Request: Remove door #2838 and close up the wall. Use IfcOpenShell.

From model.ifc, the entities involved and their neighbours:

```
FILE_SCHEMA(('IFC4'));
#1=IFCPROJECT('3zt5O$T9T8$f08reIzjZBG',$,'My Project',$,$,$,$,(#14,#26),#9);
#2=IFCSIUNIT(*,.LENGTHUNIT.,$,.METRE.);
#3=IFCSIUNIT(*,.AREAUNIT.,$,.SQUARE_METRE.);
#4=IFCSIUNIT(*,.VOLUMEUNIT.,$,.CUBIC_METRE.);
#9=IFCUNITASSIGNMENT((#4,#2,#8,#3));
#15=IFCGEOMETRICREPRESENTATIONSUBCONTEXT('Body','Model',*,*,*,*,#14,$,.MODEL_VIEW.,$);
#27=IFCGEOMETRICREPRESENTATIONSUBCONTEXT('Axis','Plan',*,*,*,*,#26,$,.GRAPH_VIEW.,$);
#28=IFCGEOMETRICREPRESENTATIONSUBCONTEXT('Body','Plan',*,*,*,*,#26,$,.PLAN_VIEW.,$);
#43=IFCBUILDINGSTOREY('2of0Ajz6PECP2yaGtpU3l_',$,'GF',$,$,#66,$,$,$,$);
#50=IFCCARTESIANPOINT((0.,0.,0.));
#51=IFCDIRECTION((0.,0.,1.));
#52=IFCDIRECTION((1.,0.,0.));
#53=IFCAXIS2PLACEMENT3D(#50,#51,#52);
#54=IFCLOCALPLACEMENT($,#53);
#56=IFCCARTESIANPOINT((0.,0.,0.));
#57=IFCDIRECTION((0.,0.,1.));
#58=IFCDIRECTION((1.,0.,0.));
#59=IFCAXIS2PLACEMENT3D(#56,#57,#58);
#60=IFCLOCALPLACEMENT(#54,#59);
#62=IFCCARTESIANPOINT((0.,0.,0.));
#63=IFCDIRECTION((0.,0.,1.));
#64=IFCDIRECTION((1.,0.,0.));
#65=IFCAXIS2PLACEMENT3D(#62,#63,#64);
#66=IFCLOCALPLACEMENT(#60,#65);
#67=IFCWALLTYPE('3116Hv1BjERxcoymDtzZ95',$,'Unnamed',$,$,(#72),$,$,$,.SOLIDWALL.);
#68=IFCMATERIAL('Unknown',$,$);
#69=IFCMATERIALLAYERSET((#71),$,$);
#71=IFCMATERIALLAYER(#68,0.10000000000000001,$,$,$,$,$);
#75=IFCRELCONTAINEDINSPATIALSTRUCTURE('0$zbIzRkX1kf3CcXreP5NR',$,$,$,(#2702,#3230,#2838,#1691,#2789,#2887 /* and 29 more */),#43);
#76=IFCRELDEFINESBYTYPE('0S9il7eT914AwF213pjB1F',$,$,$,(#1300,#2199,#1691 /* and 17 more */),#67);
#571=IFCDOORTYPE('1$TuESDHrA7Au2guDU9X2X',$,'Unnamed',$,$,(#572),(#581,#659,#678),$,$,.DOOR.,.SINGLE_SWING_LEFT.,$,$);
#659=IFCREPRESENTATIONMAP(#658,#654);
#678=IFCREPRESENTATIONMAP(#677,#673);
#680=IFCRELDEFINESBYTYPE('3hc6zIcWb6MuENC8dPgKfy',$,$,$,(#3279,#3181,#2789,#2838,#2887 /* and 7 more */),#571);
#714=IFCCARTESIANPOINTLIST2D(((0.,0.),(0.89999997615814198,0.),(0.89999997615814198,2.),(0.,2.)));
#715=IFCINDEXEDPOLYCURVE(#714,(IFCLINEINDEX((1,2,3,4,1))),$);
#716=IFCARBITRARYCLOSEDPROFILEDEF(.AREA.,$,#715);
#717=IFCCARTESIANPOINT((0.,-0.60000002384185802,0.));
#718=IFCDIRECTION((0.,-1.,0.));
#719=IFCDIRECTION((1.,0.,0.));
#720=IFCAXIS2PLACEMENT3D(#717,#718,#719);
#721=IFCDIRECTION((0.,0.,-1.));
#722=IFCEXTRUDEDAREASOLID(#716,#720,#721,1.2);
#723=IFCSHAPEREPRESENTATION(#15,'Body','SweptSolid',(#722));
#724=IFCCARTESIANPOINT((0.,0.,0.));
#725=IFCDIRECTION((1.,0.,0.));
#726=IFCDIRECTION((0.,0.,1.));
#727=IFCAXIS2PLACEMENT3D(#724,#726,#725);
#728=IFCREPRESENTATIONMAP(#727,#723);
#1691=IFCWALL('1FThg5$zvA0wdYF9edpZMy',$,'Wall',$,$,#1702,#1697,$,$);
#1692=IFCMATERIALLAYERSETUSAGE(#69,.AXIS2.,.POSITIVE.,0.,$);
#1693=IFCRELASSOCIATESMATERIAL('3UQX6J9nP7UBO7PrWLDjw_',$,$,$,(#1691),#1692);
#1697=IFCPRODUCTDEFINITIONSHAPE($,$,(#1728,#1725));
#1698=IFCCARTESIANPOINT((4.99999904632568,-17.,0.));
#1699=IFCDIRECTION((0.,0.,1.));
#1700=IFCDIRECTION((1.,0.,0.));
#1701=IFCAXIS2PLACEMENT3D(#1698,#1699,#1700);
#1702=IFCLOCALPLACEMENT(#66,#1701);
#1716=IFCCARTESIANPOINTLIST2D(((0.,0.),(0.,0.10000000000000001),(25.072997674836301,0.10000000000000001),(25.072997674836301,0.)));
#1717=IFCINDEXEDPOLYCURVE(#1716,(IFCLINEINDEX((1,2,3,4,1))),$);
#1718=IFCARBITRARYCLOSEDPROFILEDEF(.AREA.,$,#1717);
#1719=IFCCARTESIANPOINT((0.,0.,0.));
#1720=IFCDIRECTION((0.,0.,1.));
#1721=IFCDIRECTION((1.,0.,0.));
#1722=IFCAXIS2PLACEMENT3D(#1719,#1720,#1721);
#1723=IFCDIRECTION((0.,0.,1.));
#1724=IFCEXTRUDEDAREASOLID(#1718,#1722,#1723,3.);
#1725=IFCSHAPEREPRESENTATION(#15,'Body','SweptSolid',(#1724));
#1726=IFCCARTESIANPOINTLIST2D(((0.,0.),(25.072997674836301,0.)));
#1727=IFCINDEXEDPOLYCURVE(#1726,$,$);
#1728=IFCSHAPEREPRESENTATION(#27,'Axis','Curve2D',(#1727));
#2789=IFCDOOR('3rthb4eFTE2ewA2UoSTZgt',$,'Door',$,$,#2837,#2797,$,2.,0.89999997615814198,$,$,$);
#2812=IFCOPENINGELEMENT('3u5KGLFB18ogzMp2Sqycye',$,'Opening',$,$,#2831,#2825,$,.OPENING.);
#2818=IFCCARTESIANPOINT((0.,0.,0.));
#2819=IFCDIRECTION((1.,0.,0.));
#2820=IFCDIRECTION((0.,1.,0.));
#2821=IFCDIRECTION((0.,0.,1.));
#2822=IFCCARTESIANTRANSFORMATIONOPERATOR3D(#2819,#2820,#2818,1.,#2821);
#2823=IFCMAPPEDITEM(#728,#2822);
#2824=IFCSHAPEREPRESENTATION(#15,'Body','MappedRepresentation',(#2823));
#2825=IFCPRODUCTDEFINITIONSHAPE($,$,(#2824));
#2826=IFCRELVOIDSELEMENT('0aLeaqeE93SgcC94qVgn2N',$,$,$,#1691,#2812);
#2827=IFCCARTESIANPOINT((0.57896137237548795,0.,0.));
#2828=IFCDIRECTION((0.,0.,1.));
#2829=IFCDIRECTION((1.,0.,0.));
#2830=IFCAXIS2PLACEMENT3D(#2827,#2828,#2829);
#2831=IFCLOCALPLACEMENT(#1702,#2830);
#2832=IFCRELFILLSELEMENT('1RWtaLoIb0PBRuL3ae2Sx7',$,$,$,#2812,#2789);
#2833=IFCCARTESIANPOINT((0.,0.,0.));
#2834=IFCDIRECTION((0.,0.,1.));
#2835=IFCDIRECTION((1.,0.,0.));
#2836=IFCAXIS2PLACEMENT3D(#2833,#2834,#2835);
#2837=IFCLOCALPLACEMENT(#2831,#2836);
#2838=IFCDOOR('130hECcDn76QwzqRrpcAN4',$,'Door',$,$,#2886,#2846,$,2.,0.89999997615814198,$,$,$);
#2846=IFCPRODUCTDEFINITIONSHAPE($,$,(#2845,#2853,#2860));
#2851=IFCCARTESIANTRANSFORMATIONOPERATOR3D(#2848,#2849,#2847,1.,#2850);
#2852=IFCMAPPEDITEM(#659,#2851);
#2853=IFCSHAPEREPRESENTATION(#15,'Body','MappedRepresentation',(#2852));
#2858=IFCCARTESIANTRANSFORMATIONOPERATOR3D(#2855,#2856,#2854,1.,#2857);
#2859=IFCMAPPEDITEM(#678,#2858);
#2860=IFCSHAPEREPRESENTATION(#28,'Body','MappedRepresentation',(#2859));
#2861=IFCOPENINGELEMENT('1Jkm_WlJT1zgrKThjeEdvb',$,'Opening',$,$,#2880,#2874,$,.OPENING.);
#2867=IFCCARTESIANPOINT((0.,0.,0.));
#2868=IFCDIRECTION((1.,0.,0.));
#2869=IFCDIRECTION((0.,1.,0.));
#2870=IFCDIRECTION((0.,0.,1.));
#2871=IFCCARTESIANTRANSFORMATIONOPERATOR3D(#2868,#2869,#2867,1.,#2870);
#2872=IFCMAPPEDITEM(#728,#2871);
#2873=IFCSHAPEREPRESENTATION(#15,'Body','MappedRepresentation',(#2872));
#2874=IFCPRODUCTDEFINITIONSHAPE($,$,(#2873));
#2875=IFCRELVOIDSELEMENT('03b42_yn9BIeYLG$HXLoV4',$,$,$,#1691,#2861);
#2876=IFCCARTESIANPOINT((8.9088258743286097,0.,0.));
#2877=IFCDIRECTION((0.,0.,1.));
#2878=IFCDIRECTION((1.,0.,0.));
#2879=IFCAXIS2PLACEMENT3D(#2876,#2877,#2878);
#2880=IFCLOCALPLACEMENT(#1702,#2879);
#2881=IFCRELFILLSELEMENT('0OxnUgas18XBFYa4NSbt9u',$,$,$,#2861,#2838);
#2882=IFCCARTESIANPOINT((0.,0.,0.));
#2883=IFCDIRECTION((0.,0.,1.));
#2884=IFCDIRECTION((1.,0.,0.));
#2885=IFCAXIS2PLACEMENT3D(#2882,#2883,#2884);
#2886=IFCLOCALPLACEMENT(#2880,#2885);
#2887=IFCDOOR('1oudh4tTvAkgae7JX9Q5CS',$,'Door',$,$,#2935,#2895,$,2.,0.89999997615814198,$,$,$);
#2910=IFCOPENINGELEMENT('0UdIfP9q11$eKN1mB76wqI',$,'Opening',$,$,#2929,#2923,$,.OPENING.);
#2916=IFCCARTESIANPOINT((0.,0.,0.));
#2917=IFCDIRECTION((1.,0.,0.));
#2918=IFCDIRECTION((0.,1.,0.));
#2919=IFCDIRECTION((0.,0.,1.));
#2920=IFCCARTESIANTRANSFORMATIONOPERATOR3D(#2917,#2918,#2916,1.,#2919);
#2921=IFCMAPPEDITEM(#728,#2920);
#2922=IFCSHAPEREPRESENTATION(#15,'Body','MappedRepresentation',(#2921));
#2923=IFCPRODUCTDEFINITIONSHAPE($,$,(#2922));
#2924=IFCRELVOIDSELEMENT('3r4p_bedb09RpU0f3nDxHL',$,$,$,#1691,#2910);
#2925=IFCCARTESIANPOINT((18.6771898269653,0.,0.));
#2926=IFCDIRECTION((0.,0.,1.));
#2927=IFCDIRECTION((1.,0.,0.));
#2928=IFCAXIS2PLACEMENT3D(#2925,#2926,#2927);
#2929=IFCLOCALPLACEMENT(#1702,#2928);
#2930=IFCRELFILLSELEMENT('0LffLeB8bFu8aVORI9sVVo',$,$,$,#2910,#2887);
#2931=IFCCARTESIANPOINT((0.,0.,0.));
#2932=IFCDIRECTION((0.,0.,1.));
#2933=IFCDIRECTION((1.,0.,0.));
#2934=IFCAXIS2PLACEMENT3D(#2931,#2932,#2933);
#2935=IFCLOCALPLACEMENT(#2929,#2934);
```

```python
import ifcopenshell
import ifcopenshell.api.feature
import ifcopenshell.api.root
import ifcopenshell.geom
import ifcopenshell.util.shape

model = ifcopenshell.open("model.ifc")
settings = ifcopenshell.geom.settings()


def volume(element):
    """Net volume in cubic metres, openings subtracted."""
    shape = ifcopenshell.geom.create_shape(settings, element)
    return ifcopenshell.util.shape.get_volume(shape.geometry)


door = model.by_guid("130hECcDn76QwzqRrpcAN4")
opening = door.FillsVoids[0].RelatingOpeningElement
wall = opening.VoidsElements[0].RelatingBuildingElement
before = volume(wall)

ifcopenshell.api.root.remove_product(model, product=door)
ifcopenshell.api.feature.remove_feature(model, feature=opening)

after = volume(wall)

print(f"wall volume {before:.3f} -> {after:.3f} m3")

model.write("model_rev.ifc")
```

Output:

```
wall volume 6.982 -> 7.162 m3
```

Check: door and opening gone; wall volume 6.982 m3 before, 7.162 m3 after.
